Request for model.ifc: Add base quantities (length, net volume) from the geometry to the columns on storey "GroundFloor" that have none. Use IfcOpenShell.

First a look at what the model holds.

```python
import ifcopenshell
import ifcopenshell.util.element
import ifcopenshell.util.unit

model = ifcopenshell.open("model.ifc")
print(model.schema)
for unit_type in ("LENGTHUNIT", "AREAUNIT", "VOLUMEUNIT"):
    print(unit_type, ifcopenshell.util.unit.calculate_unit_scale(model, unit_type))
storey = next(s for s in model.by_type("IfcBuildingStorey") if s.Name == "GroundFloor")
columns = [e for e in ifcopenshell.util.element.get_decomposition(storey) if e.is_a("IfcColumn")]
for e in sorted(columns, key=lambda e: e.id()):
    print(e.id(), e.is_a(), e.Name, list(ifcopenshell.util.element.get_psets(e, qtos_only=True)), sep=" | ")
```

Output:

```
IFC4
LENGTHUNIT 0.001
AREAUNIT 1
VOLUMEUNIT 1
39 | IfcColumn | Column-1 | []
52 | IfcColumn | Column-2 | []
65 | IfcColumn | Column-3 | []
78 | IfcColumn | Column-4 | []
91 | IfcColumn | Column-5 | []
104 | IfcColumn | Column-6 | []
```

```python
import ifcopenshell
import ifcopenshell.api.pset
import ifcopenshell.geom
import ifcopenshell.util.element
import ifcopenshell.util.shape
import ifcopenshell.util.unit

model = ifcopenshell.open("model.ifc")
unit_scale = ifcopenshell.util.unit.calculate_unit_scale(model)
volume_scale = ifcopenshell.util.unit.calculate_unit_scale(model, "VOLUMEUNIT")
settings = ifcopenshell.geom.settings()

storey = next(s for s in model.by_type("IfcBuildingStorey") if s.Name == "GroundFloor")
columns = [e for e in ifcopenshell.util.element.get_decomposition(storey) if e.is_a("IfcColumn")]

for e in sorted(columns, key=lambda e: e.id()):
    if ifcopenshell.util.element.get_psets(e, qtos_only=True, should_inherit=False):
        continue
    # Geometry comes back in metres, in the element's own axes.
    shape = ifcopenshell.geom.create_shape(settings, e)
    values = {
        "Length": ifcopenshell.util.shape.get_z(shape.geometry) / unit_scale,
        "NetVolume": ifcopenshell.util.shape.get_volume(shape.geometry) / volume_scale,
    }
    qto = ifcopenshell.api.pset.add_qto(model, product=e, name="Qto_ColumnBaseQuantities")
    ifcopenshell.api.pset.edit_qto(model, qto=qto, properties=values)
    print(e.id(), {k: round(v, 3) for k, v in values.items()})

model.write("model-out.ifc")
```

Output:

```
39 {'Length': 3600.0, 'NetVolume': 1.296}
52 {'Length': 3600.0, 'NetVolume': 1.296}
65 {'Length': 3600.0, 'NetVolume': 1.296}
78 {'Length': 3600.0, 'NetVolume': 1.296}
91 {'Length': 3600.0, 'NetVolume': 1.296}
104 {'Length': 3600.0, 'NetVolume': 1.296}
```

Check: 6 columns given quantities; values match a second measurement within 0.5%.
